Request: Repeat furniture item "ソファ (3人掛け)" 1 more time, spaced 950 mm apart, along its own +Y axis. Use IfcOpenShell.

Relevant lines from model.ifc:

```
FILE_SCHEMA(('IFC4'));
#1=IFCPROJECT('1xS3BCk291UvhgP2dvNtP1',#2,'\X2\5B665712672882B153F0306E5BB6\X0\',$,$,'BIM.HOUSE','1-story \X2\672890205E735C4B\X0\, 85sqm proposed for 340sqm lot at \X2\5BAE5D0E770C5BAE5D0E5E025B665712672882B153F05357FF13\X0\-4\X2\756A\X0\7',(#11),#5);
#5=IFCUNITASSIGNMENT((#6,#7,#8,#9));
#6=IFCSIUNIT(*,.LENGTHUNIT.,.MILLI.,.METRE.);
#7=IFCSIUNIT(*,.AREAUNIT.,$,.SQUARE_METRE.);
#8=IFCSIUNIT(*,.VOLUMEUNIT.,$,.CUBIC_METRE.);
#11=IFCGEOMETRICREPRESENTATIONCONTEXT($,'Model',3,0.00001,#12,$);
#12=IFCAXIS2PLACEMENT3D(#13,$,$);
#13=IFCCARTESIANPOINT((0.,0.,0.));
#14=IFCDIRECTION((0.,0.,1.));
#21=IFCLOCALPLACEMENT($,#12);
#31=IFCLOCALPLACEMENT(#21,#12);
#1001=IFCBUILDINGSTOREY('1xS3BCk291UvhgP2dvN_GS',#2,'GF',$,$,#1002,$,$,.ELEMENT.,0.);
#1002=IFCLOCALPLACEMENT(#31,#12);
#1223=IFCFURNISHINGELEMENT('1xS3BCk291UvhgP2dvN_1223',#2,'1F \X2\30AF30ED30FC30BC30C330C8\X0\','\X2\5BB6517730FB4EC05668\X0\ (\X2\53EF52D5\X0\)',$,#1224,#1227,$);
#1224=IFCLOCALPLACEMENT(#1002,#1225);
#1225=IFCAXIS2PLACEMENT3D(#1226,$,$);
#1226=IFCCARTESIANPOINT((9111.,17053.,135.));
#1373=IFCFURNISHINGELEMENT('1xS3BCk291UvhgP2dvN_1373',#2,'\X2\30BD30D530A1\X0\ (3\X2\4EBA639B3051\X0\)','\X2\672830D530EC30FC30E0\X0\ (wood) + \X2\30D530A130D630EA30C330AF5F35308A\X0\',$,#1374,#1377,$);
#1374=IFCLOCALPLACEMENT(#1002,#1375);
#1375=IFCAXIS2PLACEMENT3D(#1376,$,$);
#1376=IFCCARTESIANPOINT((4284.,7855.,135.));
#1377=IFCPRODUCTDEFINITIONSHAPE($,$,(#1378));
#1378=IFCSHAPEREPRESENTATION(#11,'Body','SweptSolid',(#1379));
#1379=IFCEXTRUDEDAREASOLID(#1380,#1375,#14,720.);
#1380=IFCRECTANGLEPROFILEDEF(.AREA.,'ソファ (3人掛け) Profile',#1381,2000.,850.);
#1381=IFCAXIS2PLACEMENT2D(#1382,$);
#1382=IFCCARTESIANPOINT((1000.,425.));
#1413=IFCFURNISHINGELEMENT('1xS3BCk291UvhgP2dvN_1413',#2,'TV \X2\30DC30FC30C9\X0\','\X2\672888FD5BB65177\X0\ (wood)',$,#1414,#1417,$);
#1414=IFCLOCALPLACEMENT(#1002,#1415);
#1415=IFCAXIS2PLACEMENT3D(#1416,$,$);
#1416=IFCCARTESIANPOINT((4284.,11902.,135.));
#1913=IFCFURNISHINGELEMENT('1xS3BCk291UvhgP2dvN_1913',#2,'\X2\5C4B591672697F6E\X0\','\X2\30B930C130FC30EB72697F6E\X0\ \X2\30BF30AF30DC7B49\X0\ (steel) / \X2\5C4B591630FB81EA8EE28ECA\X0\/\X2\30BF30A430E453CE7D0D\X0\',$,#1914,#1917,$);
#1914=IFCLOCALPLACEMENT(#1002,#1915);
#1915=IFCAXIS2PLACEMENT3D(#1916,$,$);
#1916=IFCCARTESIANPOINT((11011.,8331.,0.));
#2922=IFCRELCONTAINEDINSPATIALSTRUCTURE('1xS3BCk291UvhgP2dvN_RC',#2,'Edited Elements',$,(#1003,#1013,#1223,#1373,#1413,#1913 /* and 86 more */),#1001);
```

```python
import ifcopenshell
import ifcopenshell.api.geometry
import ifcopenshell.api.root
import ifcopenshell.util.element
import ifcopenshell.util.placement

model = ifcopenshell.open("model.ifc")


def reuse_history(source, copy):
    """copy_class also copies each property set's owner history, people and application; keep the originals."""
    for rel in copy.IsDefinedBy:
        if rel.is_a("IfcRelDefinesByProperties") and (history := rel.RelatingPropertyDefinition.OwnerHistory):
            rel.RelatingPropertyDefinition.OwnerHistory = source.OwnerHistory
            ifcopenshell.util.element.remove_deep2(model, history)


source = model.by_guid("1xS3BCk291UvhgP2dvN_1373")
base = ifcopenshell.util.placement.get_local_placement(source.ObjectPlacement)
step = base[:3, 1] * 950.0

for i in range(1, 2):
    copy = ifcopenshell.api.root.copy_class(model, product=source)
    copy.Representation = ifcopenshell.util.element.copy_deep(
        model, source.Representation, exclude=["IfcGeometricRepresentationContext", "IfcRepresentationMap"]
    )
    reuse_history(source, copy)
    matrix = base.copy()
    matrix[:3, 3] += i * step
    print("added at", matrix[:3, 3].round(3) + 0.0)
    ifcopenshell.api.geometry.edit_object_placement(model, product=copy, matrix=matrix, is_si=False)

model.write("model_rev.ifc")
```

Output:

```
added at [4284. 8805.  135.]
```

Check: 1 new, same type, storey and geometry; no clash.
